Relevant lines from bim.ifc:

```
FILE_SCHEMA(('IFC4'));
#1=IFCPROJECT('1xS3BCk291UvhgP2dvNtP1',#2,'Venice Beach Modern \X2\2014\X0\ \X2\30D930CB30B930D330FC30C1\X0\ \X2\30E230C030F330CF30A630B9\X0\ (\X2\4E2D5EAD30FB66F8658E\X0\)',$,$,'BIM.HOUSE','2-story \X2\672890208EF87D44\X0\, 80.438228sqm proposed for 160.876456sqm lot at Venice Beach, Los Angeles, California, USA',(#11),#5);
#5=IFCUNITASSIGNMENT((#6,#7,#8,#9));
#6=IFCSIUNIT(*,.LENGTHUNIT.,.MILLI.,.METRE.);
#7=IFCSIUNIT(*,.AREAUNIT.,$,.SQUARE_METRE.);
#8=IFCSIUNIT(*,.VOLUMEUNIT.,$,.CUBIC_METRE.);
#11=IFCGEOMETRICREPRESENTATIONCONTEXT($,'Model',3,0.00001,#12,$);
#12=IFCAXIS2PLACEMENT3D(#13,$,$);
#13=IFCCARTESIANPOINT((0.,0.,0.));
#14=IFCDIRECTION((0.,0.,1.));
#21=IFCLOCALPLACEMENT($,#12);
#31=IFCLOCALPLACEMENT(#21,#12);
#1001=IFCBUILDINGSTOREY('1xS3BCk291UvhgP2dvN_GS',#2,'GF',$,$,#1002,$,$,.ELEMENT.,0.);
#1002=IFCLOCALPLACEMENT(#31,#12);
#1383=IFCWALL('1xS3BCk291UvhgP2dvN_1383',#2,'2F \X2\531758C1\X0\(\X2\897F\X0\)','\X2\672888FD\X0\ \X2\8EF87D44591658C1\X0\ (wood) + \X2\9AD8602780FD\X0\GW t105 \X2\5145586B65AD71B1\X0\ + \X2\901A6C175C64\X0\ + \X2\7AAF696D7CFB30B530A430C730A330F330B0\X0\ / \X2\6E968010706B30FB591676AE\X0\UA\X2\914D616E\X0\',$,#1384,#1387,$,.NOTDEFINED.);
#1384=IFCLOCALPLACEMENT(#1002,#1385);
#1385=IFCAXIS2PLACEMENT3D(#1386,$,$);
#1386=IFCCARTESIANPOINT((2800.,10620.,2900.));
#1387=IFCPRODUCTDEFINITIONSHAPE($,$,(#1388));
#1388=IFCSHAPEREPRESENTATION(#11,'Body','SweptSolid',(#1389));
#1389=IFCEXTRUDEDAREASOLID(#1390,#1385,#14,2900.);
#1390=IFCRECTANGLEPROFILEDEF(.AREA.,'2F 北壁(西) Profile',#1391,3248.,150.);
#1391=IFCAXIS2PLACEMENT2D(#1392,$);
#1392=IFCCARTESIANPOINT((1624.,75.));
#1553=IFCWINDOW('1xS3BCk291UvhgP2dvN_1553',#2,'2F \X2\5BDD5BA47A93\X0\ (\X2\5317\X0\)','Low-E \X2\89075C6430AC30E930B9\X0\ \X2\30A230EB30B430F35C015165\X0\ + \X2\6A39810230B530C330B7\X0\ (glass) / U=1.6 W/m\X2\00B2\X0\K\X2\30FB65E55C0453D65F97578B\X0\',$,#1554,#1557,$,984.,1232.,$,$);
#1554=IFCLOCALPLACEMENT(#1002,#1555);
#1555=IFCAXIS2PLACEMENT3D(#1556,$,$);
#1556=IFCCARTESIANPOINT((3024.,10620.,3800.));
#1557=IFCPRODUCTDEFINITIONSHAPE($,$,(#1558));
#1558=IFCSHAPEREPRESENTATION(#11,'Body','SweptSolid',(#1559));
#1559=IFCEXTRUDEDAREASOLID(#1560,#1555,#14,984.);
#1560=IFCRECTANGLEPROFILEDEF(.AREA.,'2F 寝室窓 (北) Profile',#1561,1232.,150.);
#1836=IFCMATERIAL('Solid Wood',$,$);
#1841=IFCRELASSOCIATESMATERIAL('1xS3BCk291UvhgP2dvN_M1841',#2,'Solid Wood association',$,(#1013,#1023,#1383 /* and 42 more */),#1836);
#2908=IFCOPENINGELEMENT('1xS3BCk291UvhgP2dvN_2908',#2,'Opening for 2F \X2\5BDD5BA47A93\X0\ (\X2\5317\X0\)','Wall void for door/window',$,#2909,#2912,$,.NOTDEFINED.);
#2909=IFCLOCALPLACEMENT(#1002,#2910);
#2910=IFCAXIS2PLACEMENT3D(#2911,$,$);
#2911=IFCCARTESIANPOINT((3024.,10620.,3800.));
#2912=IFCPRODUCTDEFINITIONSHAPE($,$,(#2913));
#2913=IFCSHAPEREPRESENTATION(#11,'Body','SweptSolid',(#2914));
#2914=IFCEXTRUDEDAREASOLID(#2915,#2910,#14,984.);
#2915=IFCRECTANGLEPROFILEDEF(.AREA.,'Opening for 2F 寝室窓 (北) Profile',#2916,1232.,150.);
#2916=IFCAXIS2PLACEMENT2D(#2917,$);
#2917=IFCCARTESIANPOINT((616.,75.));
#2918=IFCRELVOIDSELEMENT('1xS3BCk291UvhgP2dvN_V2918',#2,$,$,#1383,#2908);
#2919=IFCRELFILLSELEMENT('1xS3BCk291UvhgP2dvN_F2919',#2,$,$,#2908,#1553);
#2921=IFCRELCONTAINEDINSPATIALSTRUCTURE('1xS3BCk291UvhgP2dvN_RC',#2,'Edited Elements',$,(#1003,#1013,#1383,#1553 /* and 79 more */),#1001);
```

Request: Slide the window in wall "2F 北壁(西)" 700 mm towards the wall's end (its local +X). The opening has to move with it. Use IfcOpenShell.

```python
import ifcopenshell
import ifcopenshell.api.geometry
import ifcopenshell.util.placement
import ifcopenshell.util.unit

model = ifcopenshell.open("bim.ifc")
unit_scale = ifcopenshell.util.unit.calculate_unit_scale(model)

window = model.by_id(1553)
opening = window.FillsVoids[0].RelatingOpeningElement
wall = opening.VoidsElements[0].RelatingBuildingElement

wall_matrix = ifcopenshell.util.placement.get_local_placement(wall.ObjectPlacement)
shift = wall_matrix[:3, 0] * 0.7 / unit_scale
before = ifcopenshell.util.placement.get_local_placement(window.ObjectPlacement)[:3, 3].copy()

# The window is not placed relative to its opening, so move both.
for product in (opening, window):
    matrix = ifcopenshell.util.placement.get_local_placement(product.ObjectPlacement)
    matrix[:3, 3] += shift
    ifcopenshell.api.geometry.edit_object_placement(model, product=product, matrix=matrix, is_si=False)

after = ifcopenshell.util.placement.get_local_placement(window.ObjectPlacement)[:3, 3]
print("window moved by", (after - before).round(3) + 0.0)

model.write("bim_rev.ifc")
```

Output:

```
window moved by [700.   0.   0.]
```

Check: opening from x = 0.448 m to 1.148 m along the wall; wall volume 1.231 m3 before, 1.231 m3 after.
